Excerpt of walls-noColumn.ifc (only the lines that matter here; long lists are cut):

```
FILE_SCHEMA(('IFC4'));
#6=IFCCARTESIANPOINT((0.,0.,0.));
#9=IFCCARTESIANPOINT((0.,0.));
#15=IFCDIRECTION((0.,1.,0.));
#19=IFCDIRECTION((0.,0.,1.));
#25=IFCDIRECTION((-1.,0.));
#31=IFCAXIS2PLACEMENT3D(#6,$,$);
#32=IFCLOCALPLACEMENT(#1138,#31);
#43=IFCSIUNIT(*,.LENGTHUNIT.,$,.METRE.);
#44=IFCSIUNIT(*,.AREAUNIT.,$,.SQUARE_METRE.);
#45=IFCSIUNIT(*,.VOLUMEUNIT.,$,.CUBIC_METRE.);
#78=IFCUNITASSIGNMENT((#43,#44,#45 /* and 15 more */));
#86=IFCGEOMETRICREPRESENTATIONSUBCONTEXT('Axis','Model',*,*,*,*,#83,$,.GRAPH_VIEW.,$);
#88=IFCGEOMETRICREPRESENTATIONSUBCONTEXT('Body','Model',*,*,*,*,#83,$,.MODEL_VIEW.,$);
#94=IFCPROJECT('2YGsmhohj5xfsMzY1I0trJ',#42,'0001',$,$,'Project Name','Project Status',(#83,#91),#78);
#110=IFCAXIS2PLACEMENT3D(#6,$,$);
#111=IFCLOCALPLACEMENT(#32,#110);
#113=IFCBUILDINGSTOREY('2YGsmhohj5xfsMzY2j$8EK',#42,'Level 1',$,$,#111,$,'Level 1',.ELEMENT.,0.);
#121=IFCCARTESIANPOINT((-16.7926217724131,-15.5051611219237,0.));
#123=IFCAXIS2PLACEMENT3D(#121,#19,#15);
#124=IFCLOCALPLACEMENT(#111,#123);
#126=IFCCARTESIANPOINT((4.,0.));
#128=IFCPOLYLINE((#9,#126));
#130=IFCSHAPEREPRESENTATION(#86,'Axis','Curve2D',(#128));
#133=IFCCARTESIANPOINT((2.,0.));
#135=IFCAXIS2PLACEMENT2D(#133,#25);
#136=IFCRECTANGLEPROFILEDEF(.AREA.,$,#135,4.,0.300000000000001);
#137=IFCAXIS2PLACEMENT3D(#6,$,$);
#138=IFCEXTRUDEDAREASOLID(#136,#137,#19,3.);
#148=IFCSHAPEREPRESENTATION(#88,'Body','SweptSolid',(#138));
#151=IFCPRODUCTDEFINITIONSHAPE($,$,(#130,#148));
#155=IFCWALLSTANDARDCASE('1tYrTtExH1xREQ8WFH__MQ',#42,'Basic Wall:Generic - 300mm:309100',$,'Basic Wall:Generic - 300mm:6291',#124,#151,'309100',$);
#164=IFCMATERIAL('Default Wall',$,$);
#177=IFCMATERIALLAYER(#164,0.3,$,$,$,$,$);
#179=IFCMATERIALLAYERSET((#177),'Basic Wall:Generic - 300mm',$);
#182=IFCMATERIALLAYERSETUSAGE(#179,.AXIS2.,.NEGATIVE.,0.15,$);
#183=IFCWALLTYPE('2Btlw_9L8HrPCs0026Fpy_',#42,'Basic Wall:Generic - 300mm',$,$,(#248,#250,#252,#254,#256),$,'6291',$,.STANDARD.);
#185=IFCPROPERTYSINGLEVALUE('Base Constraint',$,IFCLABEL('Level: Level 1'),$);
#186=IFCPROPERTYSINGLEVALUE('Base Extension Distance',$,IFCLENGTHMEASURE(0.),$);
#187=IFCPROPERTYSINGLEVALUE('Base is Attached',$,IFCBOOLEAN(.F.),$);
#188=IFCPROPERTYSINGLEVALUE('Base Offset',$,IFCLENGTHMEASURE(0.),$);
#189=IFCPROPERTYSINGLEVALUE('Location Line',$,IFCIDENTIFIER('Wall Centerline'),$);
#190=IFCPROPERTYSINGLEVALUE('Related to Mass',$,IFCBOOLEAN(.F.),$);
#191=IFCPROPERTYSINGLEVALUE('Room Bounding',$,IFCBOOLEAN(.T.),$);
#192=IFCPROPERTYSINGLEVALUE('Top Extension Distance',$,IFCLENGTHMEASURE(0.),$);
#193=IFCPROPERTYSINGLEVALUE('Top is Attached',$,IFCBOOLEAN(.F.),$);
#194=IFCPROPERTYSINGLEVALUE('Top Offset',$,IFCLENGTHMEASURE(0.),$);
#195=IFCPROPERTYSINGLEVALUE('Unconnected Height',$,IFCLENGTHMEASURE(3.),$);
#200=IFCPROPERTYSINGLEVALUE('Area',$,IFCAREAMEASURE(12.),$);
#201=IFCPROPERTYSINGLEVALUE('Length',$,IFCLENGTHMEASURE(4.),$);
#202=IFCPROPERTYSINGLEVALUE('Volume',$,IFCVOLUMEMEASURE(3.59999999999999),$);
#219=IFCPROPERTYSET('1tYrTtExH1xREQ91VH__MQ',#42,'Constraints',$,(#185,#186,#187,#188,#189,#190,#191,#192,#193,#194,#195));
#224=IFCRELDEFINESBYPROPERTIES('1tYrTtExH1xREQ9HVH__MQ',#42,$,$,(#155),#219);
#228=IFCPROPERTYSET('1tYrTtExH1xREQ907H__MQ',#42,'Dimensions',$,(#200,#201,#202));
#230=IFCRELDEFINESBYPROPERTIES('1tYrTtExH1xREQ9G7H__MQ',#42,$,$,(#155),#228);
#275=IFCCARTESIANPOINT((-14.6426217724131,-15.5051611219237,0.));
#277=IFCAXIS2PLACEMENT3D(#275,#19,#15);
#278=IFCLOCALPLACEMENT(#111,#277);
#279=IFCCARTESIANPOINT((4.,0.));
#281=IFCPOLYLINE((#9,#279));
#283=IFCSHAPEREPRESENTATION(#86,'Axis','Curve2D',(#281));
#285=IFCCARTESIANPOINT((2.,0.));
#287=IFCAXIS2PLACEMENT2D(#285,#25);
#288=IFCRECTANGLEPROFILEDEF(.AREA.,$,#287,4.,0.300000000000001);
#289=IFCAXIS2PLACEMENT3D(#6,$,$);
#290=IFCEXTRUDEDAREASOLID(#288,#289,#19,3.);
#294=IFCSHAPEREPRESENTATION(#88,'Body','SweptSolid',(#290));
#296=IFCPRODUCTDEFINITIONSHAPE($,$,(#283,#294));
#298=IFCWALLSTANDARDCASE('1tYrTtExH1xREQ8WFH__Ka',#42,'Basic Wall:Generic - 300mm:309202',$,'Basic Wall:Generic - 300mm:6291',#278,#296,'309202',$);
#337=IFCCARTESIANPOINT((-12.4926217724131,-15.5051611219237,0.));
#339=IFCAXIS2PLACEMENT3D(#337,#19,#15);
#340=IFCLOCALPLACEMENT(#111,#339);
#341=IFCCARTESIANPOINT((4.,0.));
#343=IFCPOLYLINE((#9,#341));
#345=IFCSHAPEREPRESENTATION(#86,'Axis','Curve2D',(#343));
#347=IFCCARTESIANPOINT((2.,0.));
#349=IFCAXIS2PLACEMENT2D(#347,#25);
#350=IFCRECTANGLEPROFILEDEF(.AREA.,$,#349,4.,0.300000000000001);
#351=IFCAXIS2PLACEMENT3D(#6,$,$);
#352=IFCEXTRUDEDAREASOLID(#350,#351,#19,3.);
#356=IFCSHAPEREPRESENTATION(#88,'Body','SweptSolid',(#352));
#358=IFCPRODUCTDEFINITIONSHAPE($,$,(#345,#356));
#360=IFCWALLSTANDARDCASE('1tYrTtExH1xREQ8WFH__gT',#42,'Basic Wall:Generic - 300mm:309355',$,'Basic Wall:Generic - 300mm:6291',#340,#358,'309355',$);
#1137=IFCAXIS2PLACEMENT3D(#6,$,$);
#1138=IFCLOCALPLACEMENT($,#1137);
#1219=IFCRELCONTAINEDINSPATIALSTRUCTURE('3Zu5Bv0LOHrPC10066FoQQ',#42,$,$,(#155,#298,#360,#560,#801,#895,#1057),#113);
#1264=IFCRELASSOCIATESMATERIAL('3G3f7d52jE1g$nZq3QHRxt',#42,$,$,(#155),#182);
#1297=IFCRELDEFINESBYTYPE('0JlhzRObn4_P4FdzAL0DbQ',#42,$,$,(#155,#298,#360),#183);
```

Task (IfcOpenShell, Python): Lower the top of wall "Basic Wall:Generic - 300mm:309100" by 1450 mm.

```python
import ifcopenshell
import ifcopenshell.api.pset
import ifcopenshell.geom
import ifcopenshell.util.element
import ifcopenshell.util.representation
import ifcopenshell.util.shape
import ifcopenshell.util.unit

model = ifcopenshell.open("walls-noColumn.ifc")
unit_scale = ifcopenshell.util.unit.calculate_unit_scale(model)
area_scale = ifcopenshell.util.unit.calculate_unit_scale(model, "AREAUNIT")
volume_scale = ifcopenshell.util.unit.calculate_unit_scale(model, "VOLUMEUNIT")
settings = ifcopenshell.geom.settings()


def volume(element):
    """Net volume in cubic metres, openings subtracted."""
    shape = ifcopenshell.geom.create_shape(settings, element)
    return ifcopenshell.util.shape.get_volume(shape.geometry)


wall = model.by_guid("1tYrTtExH1xREQ8WFH__MQ")
before = volume(wall)

body = ifcopenshell.util.representation.get_representation(wall, "Model", "Body")
solid = body.Items[0]
old_height = solid.Depth
solid.Depth -= 1.45 / unit_scale
after = volume(wall)
thickness = 0.3  # wall thickness in metres

# Update the stored height, areas and volumes.
pset = model.by_id(ifcopenshell.util.element.get_pset(wall, "Constraints", should_inherit=False)["id"])
ifcopenshell.api.pset.edit_pset(model, pset=pset, properties={
    "Unconnected Height": model.create_entity("IfcLengthMeasure", solid.Depth),
})
pset = model.by_id(ifcopenshell.util.element.get_pset(wall, "Dimensions", should_inherit=False)["id"])
ifcopenshell.api.pset.edit_pset(model, pset=pset, properties={
    "Area": model.create_entity("IfcAreaMeasure", after / thickness / area_scale),
    "Volume": model.create_entity("IfcVolumeMeasure", after / volume_scale),
})

print(f"height {old_height:g} -> {solid.Depth:g}, volume {before:.3f} -> {after:.3f} m3")

model.write("walls-noColumn_updated.ifc")
```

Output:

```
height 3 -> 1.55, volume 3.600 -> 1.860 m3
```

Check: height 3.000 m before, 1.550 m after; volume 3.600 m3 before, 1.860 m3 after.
